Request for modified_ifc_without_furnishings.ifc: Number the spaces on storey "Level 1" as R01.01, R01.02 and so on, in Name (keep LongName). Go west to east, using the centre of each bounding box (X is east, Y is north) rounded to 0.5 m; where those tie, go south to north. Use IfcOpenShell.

First a look at what the model holds.

```python
import ifcopenshell
import ifcopenshell.util.element
import ifcopenshell.util.placement

model = ifcopenshell.open("modified_ifc_without_furnishings.ifc")
print(model.schema)
storey = next(s for s in model.by_type("IfcBuildingStorey") if s.Name == "Level 1")
spaces = [e for e in ifcopenshell.util.element.get_decomposition(storey) if e.is_a("IfcSpace")]
for e in sorted(spaces, key=lambda e: e.id()):
    origin = ifcopenshell.util.placement.get_local_placement(e.ObjectPlacement)[:3, 3]
    print(e.id(), e.Name, e.LongName, origin.round(2) + 0.0, sep=" | ")
```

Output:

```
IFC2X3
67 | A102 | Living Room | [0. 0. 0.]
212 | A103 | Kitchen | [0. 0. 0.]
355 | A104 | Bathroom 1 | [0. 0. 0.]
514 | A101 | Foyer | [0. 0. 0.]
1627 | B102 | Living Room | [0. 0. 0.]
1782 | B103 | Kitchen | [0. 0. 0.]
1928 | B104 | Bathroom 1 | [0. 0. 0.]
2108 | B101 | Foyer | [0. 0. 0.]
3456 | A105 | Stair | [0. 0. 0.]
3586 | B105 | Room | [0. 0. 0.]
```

```python
import ifcopenshell
import ifcopenshell.geom
import ifcopenshell.util.element
import ifcopenshell.util.shape

model = ifcopenshell.open("modified_ifc_without_furnishings.ifc")
settings = ifcopenshell.geom.settings()
settings.set("use-world-coords", True)


def centre(element):
    shape = ifcopenshell.geom.create_shape(settings, element)
    return ifcopenshell.util.shape.get_bbox_centroid(shape.geometry)


storey = next(s for s in model.by_type("IfcBuildingStorey") if s.Name == "Level 1")
spaces = [e for e in ifcopenshell.util.element.get_decomposition(storey) if e.is_a("IfcSpace")]

# Insertion points can sit at a corner or the storey origin, so sort by the geometry (in metres).
centres = {e: centre(e) for e in spaces}
spaces.sort(key=lambda e: (round(centres[e][0] / 0.5), centres[e][1]))

for i, e in enumerate(spaces, start=1):
    number = f"R01.{i:02d}"
    e.Name = number
    print(e.id(), number)

model.write("modified_ifc_without_furnishings_rev.ifc")
```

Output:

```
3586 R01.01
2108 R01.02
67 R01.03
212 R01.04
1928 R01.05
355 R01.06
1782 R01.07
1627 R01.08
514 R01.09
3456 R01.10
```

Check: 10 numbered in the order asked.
